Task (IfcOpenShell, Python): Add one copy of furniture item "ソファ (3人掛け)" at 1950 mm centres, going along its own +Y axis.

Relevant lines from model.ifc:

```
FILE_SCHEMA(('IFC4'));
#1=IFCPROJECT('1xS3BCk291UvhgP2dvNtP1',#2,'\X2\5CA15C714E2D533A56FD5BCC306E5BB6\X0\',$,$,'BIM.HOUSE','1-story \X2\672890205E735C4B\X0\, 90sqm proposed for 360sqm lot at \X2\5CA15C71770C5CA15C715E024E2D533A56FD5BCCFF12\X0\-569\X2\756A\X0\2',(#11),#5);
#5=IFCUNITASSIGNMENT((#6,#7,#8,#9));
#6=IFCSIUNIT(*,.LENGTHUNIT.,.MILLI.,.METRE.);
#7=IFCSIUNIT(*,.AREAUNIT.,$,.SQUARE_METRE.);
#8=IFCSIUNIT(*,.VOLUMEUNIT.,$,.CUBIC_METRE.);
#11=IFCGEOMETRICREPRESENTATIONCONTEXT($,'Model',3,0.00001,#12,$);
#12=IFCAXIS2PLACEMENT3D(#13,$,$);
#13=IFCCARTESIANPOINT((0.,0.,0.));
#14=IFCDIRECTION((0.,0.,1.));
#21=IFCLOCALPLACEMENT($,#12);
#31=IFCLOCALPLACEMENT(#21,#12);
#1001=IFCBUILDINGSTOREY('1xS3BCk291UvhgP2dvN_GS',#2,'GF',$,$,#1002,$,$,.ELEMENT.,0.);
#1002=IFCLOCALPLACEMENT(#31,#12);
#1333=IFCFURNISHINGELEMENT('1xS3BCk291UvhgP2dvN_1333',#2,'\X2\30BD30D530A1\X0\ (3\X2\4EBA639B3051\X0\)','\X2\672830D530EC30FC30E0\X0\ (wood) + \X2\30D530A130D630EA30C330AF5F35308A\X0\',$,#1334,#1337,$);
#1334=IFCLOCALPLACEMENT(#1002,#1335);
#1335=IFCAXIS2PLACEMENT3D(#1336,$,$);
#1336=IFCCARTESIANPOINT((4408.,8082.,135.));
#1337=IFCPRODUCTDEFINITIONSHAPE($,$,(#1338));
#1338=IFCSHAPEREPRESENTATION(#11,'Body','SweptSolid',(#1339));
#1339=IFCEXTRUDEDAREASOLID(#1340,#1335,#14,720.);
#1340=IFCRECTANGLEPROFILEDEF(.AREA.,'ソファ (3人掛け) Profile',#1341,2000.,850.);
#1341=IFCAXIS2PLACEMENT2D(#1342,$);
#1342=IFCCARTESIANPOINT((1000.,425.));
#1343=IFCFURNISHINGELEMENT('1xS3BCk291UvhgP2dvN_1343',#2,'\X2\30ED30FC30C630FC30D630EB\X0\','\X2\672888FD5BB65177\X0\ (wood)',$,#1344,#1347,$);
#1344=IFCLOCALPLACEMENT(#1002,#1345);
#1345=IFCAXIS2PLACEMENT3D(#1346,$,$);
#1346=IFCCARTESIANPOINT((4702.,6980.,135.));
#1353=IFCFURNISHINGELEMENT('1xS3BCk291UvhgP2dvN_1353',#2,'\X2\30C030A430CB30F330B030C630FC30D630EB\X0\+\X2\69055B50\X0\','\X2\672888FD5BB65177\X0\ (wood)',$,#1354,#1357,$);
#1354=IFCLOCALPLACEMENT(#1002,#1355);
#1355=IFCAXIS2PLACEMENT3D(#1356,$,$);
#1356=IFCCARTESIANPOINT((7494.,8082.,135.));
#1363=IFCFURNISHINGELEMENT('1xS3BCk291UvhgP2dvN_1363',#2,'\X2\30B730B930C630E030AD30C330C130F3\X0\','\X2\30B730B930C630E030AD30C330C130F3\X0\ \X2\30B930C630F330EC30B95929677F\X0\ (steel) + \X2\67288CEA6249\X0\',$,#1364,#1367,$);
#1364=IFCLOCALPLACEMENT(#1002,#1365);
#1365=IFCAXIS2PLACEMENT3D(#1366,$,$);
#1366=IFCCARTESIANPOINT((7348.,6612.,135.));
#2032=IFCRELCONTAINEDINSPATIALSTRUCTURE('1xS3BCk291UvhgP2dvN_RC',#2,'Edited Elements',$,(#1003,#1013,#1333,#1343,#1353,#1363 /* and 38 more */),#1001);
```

```python
import ifcopenshell
import ifcopenshell.api.geometry
import ifcopenshell.api.root
import ifcopenshell.util.element
import ifcopenshell.util.placement
import ifcopenshell.util.unit

model = ifcopenshell.open("model.ifc")
unit_scale = ifcopenshell.util.unit.calculate_unit_scale(model)


def reuse_history(source, copy):
    """copy_class also copies each property set's owner history, people and application; keep the originals."""
    for rel in copy.IsDefinedBy:
        if rel.is_a("IfcRelDefinesByProperties") and (history := rel.RelatingPropertyDefinition.OwnerHistory):
            rel.RelatingPropertyDefinition.OwnerHistory = source.OwnerHistory
            ifcopenshell.util.element.remove_deep2(model, history)


source = model.by_guid("1xS3BCk291UvhgP2dvN_1333")
base = ifcopenshell.util.placement.get_local_placement(source.ObjectPlacement)
step = base[:3, 1] * 1.95 / unit_scale

for i in range(1, 2):
    copy = ifcopenshell.api.root.copy_class(model, product=source)
    copy.Representation = ifcopenshell.util.element.copy_deep(
        model, source.Representation, exclude=["IfcGeometricRepresentationContext", "IfcRepresentationMap"]
    )
    reuse_history(source, copy)
    matrix = base.copy()
    matrix[:3, 3] += i * step
    print("added at", matrix[:3, 3].round(3) + 0.0)
    ifcopenshell.api.geometry.edit_object_placement(model, product=copy, matrix=matrix, is_si=False)

model.write("model_rev.ifc")
```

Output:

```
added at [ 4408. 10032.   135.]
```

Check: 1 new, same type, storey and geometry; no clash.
